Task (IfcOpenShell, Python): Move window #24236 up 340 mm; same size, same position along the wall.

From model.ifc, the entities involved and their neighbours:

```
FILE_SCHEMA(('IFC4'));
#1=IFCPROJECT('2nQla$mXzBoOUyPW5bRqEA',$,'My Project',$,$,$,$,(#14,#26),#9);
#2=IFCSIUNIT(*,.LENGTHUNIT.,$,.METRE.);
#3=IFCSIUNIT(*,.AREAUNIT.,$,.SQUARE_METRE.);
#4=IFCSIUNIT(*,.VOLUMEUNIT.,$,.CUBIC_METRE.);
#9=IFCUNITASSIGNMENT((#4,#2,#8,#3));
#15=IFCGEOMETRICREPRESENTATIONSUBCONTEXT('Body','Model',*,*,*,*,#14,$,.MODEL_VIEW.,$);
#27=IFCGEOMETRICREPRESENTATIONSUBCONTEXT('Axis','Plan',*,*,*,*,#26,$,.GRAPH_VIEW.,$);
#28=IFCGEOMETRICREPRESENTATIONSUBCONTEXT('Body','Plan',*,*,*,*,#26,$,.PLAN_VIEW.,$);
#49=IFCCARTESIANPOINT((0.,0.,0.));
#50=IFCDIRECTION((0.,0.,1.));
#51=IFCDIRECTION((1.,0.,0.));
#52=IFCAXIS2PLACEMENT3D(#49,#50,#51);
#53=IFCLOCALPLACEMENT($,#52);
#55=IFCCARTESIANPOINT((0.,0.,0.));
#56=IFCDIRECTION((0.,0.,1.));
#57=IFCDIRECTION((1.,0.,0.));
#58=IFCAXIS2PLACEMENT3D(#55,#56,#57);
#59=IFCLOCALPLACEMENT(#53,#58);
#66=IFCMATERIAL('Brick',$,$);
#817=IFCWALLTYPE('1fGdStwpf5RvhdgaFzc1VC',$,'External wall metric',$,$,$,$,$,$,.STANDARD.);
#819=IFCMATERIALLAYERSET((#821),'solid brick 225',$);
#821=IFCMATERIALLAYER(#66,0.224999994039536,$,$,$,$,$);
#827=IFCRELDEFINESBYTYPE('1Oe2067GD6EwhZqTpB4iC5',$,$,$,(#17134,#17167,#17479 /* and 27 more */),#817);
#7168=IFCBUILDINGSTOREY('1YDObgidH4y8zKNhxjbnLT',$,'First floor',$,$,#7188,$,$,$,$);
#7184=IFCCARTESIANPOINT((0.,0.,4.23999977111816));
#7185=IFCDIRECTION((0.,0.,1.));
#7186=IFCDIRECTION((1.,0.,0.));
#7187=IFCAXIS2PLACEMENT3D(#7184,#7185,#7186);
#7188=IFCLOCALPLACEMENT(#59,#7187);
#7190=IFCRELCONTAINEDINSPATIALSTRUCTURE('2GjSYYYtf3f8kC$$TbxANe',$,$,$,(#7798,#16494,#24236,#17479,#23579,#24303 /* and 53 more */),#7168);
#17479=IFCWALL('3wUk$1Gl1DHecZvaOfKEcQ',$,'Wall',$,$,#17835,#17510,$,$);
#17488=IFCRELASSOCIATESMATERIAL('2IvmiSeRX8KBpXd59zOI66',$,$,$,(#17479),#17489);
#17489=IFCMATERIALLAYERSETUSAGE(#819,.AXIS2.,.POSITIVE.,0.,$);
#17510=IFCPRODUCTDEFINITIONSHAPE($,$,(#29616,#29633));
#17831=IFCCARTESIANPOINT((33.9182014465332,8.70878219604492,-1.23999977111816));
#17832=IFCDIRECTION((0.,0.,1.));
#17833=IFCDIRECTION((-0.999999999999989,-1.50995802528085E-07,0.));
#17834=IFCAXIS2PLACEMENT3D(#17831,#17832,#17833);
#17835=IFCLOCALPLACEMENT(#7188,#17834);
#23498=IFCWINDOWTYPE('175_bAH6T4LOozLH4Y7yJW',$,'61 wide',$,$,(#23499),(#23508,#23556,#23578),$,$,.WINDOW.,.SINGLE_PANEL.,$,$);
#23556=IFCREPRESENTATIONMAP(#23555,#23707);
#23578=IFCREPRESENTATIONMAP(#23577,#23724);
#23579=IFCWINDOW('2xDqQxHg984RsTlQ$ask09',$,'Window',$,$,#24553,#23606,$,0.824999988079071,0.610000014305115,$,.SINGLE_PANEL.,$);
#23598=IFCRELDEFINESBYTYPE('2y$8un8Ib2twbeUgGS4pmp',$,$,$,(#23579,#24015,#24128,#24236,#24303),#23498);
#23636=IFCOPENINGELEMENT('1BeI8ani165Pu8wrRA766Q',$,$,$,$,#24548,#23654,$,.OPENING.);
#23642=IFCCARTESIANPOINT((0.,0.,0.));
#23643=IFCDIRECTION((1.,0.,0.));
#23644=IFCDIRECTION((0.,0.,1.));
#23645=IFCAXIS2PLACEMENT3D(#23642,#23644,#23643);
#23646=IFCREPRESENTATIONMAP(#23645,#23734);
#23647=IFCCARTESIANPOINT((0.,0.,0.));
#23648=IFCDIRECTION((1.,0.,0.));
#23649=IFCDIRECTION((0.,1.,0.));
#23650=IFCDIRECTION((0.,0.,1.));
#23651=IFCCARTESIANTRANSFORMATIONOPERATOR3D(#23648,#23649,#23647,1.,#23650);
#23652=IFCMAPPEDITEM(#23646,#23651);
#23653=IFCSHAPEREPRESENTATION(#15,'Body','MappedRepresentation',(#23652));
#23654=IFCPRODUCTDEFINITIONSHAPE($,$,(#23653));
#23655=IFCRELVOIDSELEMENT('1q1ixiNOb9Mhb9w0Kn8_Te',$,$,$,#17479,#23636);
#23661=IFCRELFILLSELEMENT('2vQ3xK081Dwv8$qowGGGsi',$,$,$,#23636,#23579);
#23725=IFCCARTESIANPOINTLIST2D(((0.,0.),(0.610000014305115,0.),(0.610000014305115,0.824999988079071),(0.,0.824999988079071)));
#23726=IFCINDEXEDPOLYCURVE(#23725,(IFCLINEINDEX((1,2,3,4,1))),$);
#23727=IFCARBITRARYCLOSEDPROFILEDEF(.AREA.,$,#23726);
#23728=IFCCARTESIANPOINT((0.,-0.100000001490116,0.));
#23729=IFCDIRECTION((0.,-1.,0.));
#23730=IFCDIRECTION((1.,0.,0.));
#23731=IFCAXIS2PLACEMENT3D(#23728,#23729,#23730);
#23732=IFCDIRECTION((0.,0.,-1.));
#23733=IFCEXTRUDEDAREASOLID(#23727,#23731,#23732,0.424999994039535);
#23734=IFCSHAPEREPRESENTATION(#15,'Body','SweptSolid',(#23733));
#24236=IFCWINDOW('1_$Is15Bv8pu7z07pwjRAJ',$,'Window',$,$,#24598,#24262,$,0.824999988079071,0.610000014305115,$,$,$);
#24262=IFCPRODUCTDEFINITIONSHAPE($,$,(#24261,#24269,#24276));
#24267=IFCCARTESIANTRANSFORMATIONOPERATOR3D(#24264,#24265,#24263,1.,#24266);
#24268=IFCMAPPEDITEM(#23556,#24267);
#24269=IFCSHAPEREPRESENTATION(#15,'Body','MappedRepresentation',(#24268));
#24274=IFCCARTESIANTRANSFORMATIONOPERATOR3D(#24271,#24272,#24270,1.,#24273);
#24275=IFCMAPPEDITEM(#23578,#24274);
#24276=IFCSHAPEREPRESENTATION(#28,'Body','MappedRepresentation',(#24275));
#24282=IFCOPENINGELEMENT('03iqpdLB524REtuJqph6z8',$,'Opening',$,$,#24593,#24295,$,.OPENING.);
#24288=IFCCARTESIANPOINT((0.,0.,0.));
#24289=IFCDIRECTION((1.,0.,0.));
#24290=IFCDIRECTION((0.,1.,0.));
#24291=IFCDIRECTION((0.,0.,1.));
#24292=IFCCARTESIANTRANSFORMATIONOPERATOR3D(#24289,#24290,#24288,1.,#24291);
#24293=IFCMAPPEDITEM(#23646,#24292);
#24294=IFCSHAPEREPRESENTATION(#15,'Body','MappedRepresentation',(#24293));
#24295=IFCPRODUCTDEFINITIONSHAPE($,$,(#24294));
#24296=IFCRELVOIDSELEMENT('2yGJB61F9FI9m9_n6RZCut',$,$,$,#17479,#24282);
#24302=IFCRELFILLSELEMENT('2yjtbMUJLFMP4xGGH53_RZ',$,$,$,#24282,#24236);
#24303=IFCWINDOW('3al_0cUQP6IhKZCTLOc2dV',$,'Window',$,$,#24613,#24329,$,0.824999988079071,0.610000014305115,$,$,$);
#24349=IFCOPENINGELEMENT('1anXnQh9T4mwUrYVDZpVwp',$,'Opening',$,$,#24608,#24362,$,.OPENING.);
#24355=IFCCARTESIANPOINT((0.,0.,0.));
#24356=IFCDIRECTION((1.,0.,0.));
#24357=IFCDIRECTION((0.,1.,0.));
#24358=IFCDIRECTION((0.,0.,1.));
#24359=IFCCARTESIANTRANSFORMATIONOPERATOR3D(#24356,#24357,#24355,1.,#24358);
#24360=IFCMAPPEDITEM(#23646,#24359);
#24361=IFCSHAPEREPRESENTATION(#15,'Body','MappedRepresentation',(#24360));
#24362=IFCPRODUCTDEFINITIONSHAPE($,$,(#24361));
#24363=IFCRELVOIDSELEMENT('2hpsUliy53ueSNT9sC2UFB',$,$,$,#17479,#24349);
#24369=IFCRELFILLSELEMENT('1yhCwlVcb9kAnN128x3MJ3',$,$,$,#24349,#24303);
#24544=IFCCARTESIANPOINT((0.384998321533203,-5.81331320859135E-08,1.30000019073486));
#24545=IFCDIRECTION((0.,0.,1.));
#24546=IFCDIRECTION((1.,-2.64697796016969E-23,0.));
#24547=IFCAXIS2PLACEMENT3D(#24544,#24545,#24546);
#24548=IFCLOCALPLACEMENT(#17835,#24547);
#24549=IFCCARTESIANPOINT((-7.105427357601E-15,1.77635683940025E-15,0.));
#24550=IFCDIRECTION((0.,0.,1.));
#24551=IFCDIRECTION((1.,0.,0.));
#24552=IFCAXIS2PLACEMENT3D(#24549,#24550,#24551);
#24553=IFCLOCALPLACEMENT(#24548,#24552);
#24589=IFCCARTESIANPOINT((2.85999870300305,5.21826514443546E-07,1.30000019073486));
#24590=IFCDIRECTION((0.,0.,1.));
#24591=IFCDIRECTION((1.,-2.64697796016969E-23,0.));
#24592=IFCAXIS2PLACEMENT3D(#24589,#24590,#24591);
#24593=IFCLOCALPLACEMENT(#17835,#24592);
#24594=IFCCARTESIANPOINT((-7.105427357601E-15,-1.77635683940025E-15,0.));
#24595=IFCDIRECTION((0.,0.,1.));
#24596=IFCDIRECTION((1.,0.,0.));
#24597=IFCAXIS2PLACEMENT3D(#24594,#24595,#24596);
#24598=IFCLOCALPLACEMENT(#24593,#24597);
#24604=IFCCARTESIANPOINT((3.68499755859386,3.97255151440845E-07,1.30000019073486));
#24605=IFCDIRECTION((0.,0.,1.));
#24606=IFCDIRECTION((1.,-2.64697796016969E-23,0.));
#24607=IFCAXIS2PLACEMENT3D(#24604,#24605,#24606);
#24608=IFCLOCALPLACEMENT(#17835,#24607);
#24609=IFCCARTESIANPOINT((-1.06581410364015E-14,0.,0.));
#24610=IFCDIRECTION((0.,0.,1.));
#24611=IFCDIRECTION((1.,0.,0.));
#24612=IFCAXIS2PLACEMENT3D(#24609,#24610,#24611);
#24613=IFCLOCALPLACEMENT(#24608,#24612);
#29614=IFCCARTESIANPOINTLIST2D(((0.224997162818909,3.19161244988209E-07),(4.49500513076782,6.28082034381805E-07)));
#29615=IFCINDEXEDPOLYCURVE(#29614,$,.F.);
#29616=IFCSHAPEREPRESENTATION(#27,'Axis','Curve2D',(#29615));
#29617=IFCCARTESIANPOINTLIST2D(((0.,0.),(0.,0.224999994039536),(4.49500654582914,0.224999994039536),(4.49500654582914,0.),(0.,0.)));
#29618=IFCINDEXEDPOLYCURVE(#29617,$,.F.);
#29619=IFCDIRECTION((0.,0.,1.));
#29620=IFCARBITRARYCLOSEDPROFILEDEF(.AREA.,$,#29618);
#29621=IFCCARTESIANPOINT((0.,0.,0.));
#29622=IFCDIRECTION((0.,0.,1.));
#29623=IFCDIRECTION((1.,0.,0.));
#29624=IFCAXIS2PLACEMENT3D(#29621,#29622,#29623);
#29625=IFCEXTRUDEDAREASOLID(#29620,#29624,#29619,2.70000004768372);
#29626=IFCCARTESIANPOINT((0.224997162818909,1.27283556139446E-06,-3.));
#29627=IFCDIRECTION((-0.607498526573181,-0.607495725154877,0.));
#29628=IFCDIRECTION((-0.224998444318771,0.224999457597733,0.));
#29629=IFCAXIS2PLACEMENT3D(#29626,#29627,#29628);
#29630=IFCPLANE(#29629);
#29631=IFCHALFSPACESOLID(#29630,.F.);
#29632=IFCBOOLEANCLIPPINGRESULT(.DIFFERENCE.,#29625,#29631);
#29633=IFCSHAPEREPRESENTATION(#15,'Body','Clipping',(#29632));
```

```python
import numpy as np
import ifcopenshell
import ifcopenshell.api.geometry
import ifcopenshell.util.placement
import ifcopenshell.util.unit

model = ifcopenshell.open("model.ifc")
unit_scale = ifcopenshell.util.unit.calculate_unit_scale(model)

window = model.by_guid("1_$Is15Bv8pu7z07pwjRAJ")
opening = window.FillsVoids[0].RelatingOpeningElement
dz = 0.34 / unit_scale

shift = np.array([0.0, 0.0, dz])
# The window is placed relative to its opening, so it follows when the opening moves.
matrix = ifcopenshell.util.placement.get_local_placement(opening.ObjectPlacement)
matrix[:3, 3] += shift
ifcopenshell.api.geometry.edit_object_placement(
    model, product=opening, matrix=matrix, is_si=False, should_transform_children=True
)

print(f"moved by {dz * unit_scale:+.3f} m")

model.write("model_updated.ifc")
```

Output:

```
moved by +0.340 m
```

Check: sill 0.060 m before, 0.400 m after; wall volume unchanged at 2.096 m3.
